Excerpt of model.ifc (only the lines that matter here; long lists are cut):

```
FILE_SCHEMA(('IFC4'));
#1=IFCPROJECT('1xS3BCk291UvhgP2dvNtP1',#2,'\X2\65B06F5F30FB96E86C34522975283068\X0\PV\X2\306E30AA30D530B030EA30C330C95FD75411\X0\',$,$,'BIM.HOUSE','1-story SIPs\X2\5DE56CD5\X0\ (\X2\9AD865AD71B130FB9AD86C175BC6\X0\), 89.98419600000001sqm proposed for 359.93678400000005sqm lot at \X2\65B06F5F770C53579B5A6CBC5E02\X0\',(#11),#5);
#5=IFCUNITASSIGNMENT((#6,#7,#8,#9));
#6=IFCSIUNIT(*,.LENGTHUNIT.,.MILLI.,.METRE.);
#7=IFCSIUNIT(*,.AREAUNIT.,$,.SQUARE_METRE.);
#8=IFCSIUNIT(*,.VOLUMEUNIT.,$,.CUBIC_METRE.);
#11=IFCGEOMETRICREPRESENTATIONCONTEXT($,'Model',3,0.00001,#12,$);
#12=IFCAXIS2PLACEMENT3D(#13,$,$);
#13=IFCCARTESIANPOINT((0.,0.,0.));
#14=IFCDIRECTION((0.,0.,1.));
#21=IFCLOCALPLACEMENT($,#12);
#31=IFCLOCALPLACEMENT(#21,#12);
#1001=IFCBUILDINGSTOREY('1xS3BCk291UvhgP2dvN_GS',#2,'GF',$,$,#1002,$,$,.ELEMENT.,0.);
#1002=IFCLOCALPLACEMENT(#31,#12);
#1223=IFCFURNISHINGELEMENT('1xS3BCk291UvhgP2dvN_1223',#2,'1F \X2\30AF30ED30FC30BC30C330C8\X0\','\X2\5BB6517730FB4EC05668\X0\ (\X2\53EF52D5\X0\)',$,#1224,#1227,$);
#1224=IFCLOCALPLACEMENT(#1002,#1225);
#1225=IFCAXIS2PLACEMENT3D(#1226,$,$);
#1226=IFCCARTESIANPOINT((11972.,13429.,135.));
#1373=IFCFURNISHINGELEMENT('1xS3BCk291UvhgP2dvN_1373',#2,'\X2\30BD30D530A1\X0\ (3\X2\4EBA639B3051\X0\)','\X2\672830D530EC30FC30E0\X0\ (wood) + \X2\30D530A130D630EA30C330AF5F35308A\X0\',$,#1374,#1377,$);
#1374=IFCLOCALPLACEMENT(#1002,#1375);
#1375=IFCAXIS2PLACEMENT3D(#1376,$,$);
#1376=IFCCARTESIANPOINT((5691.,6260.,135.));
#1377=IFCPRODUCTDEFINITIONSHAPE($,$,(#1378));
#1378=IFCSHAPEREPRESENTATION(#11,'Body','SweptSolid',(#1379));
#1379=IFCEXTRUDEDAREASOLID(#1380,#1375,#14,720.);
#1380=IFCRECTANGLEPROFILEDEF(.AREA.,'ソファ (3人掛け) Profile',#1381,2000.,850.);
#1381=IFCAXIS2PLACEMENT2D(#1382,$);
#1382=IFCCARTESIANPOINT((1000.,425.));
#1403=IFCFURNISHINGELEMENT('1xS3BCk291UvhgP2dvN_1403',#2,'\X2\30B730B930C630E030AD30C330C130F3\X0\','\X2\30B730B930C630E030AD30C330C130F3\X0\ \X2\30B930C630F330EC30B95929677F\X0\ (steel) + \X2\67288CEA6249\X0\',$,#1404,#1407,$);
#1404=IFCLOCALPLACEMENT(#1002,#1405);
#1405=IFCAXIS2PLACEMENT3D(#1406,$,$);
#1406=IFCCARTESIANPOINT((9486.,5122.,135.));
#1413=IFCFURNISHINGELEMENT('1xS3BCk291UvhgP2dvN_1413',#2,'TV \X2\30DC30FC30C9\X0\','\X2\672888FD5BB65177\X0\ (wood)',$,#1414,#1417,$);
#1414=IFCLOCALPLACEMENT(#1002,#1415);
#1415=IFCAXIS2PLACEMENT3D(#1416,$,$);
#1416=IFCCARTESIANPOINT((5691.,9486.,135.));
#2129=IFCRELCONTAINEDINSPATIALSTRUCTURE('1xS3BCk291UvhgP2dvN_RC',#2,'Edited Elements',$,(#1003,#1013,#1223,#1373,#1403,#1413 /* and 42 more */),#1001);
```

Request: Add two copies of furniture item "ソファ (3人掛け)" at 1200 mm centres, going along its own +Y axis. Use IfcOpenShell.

```python
import ifcopenshell
import ifcopenshell.api.geometry
import ifcopenshell.api.root
import ifcopenshell.util.element
import ifcopenshell.util.placement

model = ifcopenshell.open("model.ifc")


def reuse_history(source, copy):
    """copy_class also copies each property set's owner history, people and application; keep the originals."""
    for rel in copy.IsDefinedBy:
        if rel.is_a("IfcRelDefinesByProperties") and (history := rel.RelatingPropertyDefinition.OwnerHistory):
            rel.RelatingPropertyDefinition.OwnerHistory = source.OwnerHistory
            ifcopenshell.util.element.remove_deep2(model, history)


source = model.by_guid("1xS3BCk291UvhgP2dvN_1373")
base = ifcopenshell.util.placement.get_local_placement(source.ObjectPlacement)
step = base[:3, 1] * 1200.0

for i in range(1, 3):
    copy = ifcopenshell.api.root.copy_class(model, product=source)
    copy.Representation = ifcopenshell.util.element.copy_deep(
        model, source.Representation, exclude=["IfcGeometricRepresentationContext", "IfcRepresentationMap"]
    )
    reuse_history(source, copy)
    matrix = base.copy()
    matrix[:3, 3] += i * step
    print("added at", matrix[:3, 3].round(3) + 0.0)
    ifcopenshell.api.geometry.edit_object_placement(model, product=copy, matrix=matrix, is_si=False)

model.write("model_updated.ifc")
```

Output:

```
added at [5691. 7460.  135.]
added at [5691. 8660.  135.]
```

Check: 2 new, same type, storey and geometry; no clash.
